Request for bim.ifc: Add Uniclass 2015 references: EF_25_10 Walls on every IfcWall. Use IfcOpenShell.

First a look at what the model holds.

```python
import ifcopenshell

model = ifcopenshell.open("bim.ifc")
print(model.schema)
print("classifications:", [c.Name for c in model.by_type("IfcClassification")])
for ifc_class in ("IfcDoor", "IfcRoof", "IfcStair", "IfcWall", "IfcWindow"):
    print(ifc_class, len(model.by_type(ifc_class)))
```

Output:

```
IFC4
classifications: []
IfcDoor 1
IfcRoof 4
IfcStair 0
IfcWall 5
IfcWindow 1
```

```python
import ifcopenshell
import ifcopenshell.api.classification

model = ifcopenshell.open("bim.ifc")

system = ifcopenshell.api.classification.add_classification(model, classification="Uniclass 2015")

codes = {
    "IfcWall": ("EF_25_10", "Walls"),
}
for ifc_class, (code, name) in codes.items():
    products = model.by_type(ifc_class)
    ifcopenshell.api.classification.add_reference(
        model, products=products, classification=system, identification=code, name=name
    )
    print(code, len(products))

model.write("bim_updated.ifc")
```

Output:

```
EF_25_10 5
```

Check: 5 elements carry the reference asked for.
